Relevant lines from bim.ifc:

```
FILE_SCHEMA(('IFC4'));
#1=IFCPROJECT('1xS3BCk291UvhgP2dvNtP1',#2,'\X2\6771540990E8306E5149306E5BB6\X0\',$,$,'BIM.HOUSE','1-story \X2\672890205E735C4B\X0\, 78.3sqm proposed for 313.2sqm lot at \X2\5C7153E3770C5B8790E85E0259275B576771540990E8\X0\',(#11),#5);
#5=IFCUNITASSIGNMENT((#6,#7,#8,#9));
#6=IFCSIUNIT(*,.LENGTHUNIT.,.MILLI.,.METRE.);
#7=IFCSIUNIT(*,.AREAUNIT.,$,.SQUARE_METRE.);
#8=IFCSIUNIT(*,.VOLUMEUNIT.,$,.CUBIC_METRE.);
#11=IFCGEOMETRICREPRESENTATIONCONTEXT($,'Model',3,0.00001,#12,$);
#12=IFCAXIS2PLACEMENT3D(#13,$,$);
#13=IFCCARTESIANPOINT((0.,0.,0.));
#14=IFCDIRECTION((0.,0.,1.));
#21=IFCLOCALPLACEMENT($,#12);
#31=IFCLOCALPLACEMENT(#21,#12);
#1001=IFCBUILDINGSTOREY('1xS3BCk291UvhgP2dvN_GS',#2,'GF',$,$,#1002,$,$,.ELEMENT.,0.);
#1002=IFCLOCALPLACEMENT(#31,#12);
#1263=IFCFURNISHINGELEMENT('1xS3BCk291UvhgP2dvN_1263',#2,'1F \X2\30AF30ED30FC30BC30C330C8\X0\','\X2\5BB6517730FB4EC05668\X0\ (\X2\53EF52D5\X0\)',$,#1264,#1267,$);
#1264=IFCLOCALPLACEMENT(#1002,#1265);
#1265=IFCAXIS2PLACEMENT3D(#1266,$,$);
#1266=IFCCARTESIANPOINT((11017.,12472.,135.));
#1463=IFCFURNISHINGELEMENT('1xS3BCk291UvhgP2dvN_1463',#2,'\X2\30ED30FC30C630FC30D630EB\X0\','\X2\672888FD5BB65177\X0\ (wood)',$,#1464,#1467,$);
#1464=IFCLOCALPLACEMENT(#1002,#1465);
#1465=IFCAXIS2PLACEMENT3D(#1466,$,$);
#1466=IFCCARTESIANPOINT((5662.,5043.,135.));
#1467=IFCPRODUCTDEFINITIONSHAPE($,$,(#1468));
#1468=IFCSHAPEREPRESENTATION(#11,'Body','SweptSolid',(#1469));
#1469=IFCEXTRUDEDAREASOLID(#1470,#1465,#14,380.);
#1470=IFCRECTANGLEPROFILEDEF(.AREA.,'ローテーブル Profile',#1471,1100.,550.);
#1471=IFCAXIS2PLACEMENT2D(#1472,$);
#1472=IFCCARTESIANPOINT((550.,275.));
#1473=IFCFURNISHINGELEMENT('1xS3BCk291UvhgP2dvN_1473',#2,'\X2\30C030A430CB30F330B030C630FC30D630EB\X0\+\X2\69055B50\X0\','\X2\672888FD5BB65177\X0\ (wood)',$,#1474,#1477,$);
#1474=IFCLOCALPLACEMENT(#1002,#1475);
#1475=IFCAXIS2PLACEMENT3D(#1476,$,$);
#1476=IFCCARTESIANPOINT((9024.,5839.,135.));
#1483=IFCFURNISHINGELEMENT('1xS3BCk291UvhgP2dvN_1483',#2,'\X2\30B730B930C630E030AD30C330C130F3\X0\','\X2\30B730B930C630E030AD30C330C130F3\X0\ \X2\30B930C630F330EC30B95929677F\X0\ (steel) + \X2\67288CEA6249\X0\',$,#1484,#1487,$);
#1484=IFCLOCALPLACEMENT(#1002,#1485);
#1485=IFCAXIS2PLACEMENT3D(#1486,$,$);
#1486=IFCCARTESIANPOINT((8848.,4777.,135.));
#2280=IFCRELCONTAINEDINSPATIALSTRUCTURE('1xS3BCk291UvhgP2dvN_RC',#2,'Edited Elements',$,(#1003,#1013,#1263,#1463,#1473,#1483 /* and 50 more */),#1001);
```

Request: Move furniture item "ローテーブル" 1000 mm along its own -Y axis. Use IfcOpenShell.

```python
import ifcopenshell
import ifcopenshell.api.geometry
import ifcopenshell.util.placement

model = ifcopenshell.open("bim.ifc")

item = model.by_guid("1xS3BCk291UvhgP2dvN_1463")
matrix = ifcopenshell.util.placement.get_local_placement(item.ObjectPlacement)
matrix[:3, 3] -= matrix[:3, 1] * 1000.0
ifcopenshell.api.geometry.edit_object_placement(model, product=item, matrix=matrix, is_si=False)

print(ifcopenshell.util.placement.get_local_placement(item.ObjectPlacement).round(3) + 0.0)

model.write("bim_rev.ifc")
```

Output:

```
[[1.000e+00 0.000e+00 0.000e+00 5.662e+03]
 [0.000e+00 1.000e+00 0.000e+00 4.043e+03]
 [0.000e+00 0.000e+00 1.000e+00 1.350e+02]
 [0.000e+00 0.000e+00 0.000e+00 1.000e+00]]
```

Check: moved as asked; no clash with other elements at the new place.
